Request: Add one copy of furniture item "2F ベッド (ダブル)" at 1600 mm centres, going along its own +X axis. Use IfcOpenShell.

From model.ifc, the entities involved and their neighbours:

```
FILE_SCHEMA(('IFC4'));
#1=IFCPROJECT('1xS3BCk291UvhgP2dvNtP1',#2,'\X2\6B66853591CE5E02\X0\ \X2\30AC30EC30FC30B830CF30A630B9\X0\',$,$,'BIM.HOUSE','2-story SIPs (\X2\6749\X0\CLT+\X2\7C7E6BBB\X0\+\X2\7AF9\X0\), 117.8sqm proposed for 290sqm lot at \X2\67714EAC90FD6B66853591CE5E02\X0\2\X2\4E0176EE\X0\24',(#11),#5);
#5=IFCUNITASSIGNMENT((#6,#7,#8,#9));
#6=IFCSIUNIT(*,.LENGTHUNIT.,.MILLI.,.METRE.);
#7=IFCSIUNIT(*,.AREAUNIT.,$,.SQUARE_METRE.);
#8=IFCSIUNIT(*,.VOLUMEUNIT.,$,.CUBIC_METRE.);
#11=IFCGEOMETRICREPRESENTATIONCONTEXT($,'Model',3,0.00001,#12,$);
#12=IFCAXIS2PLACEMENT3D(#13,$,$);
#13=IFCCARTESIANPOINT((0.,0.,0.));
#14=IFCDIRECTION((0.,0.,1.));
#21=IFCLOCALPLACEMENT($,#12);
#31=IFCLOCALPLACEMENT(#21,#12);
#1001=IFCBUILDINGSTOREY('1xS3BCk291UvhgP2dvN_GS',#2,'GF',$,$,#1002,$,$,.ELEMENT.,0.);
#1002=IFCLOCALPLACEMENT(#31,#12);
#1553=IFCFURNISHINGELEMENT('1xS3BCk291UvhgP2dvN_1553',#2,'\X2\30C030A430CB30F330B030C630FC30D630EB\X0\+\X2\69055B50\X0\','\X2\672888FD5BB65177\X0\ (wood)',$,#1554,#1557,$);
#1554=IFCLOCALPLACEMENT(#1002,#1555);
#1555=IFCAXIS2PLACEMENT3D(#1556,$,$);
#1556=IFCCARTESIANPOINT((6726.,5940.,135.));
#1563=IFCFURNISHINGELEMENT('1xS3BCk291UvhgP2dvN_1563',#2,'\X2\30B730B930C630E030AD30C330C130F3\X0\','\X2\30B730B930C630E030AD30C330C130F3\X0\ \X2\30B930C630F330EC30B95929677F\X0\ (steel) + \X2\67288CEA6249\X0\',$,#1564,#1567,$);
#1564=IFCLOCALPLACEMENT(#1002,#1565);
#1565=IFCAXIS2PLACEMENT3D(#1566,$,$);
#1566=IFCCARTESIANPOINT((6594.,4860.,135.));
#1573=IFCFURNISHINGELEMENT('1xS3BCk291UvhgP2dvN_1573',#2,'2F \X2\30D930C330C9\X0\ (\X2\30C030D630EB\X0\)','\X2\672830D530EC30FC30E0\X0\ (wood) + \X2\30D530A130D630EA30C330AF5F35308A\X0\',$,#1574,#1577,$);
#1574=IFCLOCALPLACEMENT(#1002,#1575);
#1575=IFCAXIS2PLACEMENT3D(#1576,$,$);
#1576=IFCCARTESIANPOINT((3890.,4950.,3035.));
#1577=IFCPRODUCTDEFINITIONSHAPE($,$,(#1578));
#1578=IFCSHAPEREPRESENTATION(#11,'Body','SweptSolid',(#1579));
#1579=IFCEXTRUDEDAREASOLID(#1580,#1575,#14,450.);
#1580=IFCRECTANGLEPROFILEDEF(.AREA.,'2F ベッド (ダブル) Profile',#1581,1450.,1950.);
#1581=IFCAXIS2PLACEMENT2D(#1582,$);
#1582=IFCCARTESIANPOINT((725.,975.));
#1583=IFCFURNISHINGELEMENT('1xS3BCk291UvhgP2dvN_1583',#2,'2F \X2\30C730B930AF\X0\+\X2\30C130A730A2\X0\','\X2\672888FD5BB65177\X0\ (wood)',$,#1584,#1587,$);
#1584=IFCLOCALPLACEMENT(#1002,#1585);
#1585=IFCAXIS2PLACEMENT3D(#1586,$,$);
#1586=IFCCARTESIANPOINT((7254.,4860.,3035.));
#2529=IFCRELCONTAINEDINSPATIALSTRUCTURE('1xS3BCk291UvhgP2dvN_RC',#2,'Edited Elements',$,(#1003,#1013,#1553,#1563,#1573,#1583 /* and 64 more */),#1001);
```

```python
import ifcopenshell
import ifcopenshell.api.geometry
import ifcopenshell.api.root
import ifcopenshell.util.element
import ifcopenshell.util.placement
import ifcopenshell.util.unit

model = ifcopenshell.open("model.ifc")
unit_scale = ifcopenshell.util.unit.calculate_unit_scale(model)


def reuse_history(source, copy):
    """copy_class also copies each property set's owner history, people and application; keep the originals."""
    for rel in copy.IsDefinedBy:
        if rel.is_a("IfcRelDefinesByProperties") and (history := rel.RelatingPropertyDefinition.OwnerHistory):
            rel.RelatingPropertyDefinition.OwnerHistory = source.OwnerHistory
            ifcopenshell.util.element.remove_deep2(model, history)


source = model.by_guid("1xS3BCk291UvhgP2dvN_1573")
base = ifcopenshell.util.placement.get_local_placement(source.ObjectPlacement)
step = base[:3, 0] * 1.6 / unit_scale

for i in range(1, 2):
    copy = ifcopenshell.api.root.copy_class(model, product=source)
    copy.Representation = ifcopenshell.util.element.copy_deep(
        model, source.Representation, exclude=["IfcGeometricRepresentationContext", "IfcRepresentationMap"]
    )
    reuse_history(source, copy)
    matrix = base.copy()
    matrix[:3, 3] += i * step
    print("added at", matrix[:3, 3].round(3) + 0.0)
    ifcopenshell.api.geometry.edit_object_placement(model, product=copy, matrix=matrix, is_si=False)

model.write("model_updated.ifc")
```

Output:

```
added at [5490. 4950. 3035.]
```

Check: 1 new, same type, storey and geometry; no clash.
